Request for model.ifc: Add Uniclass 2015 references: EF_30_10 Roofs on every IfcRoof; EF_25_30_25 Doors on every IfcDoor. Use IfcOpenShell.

First a look at what the model holds.

```python
import ifcopenshell

model = ifcopenshell.open("model.ifc")
print(model.schema)
print("classifications:", [c.Name for c in model.by_type("IfcClassification")])
for ifc_class in ("IfcDoor", "IfcRoof", "IfcStair", "IfcWall", "IfcWindow"):
    print(ifc_class, len(model.by_type(ifc_class)))
```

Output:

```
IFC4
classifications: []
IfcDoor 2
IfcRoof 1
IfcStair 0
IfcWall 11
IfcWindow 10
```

```python
import ifcopenshell
import ifcopenshell.api.classification

model = ifcopenshell.open("model.ifc")

system = ifcopenshell.api.classification.add_classification(model, classification="Uniclass 2015")

codes = {
    "IfcRoof": ("EF_30_10", "Roofs"),
    "IfcDoor": ("EF_25_30_25", "Doors"),
}
for ifc_class, (code, name) in codes.items():
    products = model.by_type(ifc_class)
    ifcopenshell.api.classification.add_reference(
        model, products=products, classification=system, identification=code, name=name
    )
    print(code, len(products))

model.write("model-out.ifc")
```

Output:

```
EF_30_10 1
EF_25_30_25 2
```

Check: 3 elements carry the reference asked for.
